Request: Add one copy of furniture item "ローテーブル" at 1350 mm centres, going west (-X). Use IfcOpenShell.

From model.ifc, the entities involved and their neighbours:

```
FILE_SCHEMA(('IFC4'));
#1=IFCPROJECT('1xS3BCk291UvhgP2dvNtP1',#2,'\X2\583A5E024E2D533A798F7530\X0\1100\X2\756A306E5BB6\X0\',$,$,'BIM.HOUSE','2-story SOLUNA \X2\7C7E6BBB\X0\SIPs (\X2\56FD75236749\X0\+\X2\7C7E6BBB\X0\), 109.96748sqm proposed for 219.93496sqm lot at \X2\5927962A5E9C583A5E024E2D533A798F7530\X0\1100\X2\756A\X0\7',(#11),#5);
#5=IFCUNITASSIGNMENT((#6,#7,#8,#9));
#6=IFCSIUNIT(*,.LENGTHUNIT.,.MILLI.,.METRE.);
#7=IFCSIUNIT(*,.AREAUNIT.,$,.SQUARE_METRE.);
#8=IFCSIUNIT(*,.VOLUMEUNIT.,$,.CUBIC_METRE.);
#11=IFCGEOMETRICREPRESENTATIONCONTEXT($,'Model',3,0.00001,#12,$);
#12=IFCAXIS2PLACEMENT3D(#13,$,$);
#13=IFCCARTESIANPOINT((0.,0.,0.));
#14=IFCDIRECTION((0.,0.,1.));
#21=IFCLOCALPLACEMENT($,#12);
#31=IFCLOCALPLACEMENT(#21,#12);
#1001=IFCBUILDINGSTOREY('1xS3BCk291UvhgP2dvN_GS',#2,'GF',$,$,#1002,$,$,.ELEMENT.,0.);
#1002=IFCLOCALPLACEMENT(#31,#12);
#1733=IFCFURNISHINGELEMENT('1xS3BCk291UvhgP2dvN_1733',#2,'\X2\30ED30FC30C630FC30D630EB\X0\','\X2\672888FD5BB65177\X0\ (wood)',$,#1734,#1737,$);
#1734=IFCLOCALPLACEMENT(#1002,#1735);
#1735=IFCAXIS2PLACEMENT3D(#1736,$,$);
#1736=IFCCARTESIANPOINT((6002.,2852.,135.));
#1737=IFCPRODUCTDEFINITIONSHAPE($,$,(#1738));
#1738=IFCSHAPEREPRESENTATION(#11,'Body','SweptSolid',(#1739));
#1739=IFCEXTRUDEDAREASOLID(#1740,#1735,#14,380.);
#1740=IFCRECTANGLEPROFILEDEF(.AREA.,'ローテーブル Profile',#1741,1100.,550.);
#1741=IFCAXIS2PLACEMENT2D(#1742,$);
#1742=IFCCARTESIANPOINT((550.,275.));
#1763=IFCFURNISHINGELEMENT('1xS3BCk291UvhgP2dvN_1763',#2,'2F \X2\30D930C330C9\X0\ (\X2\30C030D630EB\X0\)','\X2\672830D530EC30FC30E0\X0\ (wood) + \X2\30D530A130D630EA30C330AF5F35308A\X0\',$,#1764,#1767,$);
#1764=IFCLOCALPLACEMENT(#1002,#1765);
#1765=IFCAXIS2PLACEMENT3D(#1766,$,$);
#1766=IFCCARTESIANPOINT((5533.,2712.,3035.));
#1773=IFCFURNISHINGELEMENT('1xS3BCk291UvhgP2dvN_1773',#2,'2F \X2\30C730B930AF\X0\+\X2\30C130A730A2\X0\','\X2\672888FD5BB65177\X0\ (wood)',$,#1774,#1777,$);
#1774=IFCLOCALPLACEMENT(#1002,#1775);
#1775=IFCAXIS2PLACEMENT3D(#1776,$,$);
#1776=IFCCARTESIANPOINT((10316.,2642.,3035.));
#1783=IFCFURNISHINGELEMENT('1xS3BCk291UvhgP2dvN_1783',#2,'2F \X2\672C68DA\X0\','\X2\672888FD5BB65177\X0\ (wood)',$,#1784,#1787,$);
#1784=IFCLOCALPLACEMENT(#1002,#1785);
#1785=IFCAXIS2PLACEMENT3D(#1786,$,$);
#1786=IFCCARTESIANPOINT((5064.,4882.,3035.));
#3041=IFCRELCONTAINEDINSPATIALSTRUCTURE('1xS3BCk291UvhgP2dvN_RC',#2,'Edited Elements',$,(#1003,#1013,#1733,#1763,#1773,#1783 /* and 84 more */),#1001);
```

```python
import numpy as np
import ifcopenshell
import ifcopenshell.api.geometry
import ifcopenshell.api.root
import ifcopenshell.util.element
import ifcopenshell.util.placement
import ifcopenshell.util.unit

model = ifcopenshell.open("model.ifc")
unit_scale = ifcopenshell.util.unit.calculate_unit_scale(model)


def reuse_history(source, copy):
    """copy_class also copies each property set's owner history, people and application; keep the originals."""
    for rel in copy.IsDefinedBy:
        if rel.is_a("IfcRelDefinesByProperties") and (history := rel.RelatingPropertyDefinition.OwnerHistory):
            rel.RelatingPropertyDefinition.OwnerHistory = source.OwnerHistory
            ifcopenshell.util.element.remove_deep2(model, history)


source = model.by_guid("1xS3BCk291UvhgP2dvN_1733")
base = ifcopenshell.util.placement.get_local_placement(source.ObjectPlacement)
step = np.array([-1.0, 0.0, 0.0]) * 1.35 / unit_scale

for i in range(1, 2):
    copy = ifcopenshell.api.root.copy_class(model, product=source)
    copy.Representation = ifcopenshell.util.element.copy_deep(
        model, source.Representation, exclude=["IfcGeometricRepresentationContext", "IfcRepresentationMap"]
    )
    reuse_history(source, copy)
    matrix = base.copy()
    matrix[:3, 3] += i * step
    print("added at", matrix[:3, 3].round(3) + 0.0)
    ifcopenshell.api.geometry.edit_object_placement(model, product=copy, matrix=matrix, is_si=False)

model.write("model_rev.ifc")
```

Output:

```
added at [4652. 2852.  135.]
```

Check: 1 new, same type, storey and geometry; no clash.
